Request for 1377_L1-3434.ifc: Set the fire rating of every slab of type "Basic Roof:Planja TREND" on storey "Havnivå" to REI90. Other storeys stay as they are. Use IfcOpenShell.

First a look at what the model holds.

```python
import ifcopenshell
import ifcopenshell.util.element

model = ifcopenshell.open("1377_L1-3434.ifc")
print(model.schema)
storey = next(s for s in model.by_type("IfcBuildingStorey") if s.Name == "Havnivå")
slabs = [e for e in ifcopenshell.util.element.get_decomposition(storey) if e.is_a("IfcSlab")]
seen = {}
for e in slabs:
    element_type = ifcopenshell.util.element.get_type(e)
    key = (element_type.Name if element_type != e and element_type else None, ifcopenshell.util.element.get_pset(e, "Pset_SlabCommon", "FireRating"))
    seen[key] = seen.get(key, 0) + 1
for (name, value), count in sorted(seen.items(), key=str):
    print(count, "x", name, "|", value)
```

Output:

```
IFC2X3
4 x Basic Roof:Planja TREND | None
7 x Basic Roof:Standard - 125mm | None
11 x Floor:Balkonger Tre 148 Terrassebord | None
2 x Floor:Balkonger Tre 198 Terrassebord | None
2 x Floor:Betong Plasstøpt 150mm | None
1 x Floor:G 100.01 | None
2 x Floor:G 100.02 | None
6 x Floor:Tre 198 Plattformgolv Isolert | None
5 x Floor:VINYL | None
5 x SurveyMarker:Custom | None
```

```python
import ifcopenshell
import ifcopenshell.api.pset
import ifcopenshell.util.element

model = ifcopenshell.open("1377_L1-3434.ifc")

storey = next(s for s in model.by_type("IfcBuildingStorey") if s.Name == "Havnivå")
slabs = [e for e in ifcopenshell.util.element.get_decomposition(storey) if e.is_a("IfcSlab")]

count = 0
for e in slabs:
    element_type = ifcopenshell.util.element.get_type(e)
    if element_type in (None, e) or element_type.Name != "Basic Roof:Planja TREND":
        continue
    # add_pset returns the element's existing set when there is one.
    pset = ifcopenshell.api.pset.add_pset(model, product=e, name="Pset_SlabCommon")
    ifcopenshell.api.pset.edit_pset(model, pset=pset, properties={"FireRating": "REI90"})
    count += 1

print(count, "slabs updated")

model.write("1377_L1-3434_rev.ifc")
```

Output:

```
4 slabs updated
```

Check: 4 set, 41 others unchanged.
